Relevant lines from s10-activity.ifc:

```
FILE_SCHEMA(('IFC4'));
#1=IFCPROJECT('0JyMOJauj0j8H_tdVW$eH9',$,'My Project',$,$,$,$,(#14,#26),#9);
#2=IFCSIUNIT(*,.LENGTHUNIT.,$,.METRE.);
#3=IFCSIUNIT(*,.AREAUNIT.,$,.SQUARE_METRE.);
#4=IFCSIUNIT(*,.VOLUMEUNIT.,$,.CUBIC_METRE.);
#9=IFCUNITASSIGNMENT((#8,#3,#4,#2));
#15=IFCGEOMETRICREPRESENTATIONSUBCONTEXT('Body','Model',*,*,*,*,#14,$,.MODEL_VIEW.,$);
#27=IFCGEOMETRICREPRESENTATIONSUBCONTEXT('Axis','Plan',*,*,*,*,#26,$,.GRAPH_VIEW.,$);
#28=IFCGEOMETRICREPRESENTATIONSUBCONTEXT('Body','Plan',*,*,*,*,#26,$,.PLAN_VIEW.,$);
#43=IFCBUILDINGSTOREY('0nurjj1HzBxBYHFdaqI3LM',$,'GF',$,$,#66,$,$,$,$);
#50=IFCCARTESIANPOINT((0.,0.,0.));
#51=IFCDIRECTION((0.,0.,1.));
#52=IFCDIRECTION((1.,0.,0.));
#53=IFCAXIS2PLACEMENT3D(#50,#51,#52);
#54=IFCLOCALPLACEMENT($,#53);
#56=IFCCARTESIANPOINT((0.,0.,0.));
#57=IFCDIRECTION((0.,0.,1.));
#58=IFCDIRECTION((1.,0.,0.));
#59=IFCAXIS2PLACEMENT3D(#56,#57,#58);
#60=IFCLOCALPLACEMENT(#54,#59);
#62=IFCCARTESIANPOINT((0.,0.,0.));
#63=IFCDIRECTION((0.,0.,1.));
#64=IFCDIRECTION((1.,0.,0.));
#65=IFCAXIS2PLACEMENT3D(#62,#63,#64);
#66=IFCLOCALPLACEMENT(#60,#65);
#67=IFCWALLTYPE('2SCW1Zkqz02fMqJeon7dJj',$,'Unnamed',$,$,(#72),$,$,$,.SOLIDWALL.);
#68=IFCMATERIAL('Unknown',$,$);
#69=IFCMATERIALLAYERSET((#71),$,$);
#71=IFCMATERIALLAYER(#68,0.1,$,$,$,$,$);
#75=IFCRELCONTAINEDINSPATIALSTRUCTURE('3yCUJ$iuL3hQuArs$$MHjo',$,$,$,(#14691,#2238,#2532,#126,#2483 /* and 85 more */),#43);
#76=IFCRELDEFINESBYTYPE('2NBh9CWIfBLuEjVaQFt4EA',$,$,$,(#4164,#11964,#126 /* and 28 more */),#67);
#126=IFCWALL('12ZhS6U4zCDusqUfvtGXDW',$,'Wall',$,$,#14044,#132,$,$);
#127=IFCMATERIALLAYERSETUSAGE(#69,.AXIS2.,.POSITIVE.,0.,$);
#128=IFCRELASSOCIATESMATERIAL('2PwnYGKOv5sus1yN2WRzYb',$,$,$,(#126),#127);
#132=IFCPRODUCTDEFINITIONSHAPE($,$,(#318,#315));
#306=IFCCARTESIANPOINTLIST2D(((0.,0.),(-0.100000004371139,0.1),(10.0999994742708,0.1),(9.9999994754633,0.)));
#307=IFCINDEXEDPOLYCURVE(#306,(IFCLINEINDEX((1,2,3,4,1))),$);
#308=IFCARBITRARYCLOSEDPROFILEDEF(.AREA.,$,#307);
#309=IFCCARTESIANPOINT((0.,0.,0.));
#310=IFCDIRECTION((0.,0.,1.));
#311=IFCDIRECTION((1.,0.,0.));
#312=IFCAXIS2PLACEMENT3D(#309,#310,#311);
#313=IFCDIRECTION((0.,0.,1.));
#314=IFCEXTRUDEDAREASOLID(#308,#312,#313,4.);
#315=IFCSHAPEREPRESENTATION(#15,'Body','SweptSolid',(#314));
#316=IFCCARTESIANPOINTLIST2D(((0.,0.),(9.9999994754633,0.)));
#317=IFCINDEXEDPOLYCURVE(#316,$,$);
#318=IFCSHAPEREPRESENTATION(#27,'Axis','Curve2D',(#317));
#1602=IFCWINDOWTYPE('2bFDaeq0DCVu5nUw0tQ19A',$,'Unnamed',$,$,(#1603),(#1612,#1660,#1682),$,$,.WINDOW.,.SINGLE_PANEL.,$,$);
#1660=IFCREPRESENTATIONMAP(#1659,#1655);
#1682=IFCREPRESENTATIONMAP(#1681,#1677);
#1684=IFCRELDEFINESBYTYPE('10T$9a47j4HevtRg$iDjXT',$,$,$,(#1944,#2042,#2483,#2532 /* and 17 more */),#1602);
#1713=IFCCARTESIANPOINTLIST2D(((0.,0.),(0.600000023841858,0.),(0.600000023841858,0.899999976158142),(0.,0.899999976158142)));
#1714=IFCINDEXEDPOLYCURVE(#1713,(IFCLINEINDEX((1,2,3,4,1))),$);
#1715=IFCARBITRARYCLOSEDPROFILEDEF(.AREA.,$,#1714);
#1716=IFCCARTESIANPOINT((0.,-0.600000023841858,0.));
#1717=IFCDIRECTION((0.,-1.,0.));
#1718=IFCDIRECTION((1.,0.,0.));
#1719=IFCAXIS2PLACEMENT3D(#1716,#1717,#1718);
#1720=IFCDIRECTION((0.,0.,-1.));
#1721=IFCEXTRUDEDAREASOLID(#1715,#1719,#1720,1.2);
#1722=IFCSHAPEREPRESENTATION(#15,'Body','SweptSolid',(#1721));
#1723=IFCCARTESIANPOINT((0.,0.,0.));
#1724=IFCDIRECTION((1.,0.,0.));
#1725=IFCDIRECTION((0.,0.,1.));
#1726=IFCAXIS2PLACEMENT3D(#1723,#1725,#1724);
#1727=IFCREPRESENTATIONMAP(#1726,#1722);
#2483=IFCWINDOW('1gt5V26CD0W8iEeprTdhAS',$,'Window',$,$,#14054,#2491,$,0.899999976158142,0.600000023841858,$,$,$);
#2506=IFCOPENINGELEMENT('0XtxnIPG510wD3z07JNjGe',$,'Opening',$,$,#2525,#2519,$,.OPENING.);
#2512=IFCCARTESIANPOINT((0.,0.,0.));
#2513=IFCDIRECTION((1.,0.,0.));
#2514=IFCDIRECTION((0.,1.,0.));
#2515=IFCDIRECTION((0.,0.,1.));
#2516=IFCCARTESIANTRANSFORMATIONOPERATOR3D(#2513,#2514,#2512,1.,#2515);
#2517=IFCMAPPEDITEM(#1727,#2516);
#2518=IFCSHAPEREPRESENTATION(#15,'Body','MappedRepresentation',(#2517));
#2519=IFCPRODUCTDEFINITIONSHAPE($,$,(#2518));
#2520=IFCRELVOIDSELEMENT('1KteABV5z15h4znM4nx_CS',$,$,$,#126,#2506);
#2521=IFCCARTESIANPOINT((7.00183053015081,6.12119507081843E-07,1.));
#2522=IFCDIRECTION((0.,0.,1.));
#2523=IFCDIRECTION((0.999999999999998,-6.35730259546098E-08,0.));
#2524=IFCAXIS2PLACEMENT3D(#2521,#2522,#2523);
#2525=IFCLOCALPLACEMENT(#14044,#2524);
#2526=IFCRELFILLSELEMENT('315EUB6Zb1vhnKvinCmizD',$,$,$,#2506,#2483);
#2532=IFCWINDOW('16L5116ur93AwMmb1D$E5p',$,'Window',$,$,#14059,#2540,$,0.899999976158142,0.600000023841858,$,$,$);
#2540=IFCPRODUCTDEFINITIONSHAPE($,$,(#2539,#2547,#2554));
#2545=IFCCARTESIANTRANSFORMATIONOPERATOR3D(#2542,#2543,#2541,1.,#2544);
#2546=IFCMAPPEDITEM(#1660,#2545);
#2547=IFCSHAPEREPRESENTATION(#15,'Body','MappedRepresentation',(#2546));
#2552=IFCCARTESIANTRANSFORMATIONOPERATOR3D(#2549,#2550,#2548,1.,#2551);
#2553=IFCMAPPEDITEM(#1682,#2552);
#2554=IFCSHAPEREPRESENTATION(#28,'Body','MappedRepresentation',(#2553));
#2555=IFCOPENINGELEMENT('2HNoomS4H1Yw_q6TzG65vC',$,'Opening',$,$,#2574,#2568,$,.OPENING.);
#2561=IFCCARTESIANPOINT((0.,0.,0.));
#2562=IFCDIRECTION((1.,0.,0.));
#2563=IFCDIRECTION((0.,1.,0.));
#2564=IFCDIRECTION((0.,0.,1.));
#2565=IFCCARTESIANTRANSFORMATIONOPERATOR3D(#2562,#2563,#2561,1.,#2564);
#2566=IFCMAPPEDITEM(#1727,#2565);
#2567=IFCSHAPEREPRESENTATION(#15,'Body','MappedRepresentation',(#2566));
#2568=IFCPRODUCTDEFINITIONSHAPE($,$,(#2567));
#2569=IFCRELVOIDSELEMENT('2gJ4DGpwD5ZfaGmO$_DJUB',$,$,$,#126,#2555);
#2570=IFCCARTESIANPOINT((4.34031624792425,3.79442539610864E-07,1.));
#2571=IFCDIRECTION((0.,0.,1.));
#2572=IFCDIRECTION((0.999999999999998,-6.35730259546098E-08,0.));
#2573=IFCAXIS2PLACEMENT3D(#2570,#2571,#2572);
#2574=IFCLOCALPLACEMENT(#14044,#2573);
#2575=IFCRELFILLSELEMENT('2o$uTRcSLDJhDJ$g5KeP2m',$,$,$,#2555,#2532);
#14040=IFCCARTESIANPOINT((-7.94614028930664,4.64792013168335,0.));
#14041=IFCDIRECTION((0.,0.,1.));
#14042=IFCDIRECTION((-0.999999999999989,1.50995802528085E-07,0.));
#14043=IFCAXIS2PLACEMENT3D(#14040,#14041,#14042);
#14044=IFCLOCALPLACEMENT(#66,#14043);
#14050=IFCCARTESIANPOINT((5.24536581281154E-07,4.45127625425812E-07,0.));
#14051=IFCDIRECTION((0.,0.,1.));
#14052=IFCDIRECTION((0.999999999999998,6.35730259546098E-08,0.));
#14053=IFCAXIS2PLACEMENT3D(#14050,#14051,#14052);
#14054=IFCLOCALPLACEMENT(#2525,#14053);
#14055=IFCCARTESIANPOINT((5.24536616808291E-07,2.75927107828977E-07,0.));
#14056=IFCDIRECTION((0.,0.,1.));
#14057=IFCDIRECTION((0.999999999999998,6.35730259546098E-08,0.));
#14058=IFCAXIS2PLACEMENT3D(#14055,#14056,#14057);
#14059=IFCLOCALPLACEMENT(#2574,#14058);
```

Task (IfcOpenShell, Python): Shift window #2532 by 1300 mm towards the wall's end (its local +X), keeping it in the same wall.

```python
import ifcopenshell
import ifcopenshell.api.geometry
import ifcopenshell.util.placement

model = ifcopenshell.open("s10-activity.ifc")

window = model.by_id(2532)
opening = window.FillsVoids[0].RelatingOpeningElement
wall = opening.VoidsElements[0].RelatingBuildingElement

wall_matrix = ifcopenshell.util.placement.get_local_placement(wall.ObjectPlacement)
shift = wall_matrix[:3, 0] * 1.3
before = ifcopenshell.util.placement.get_local_placement(window.ObjectPlacement)[:3, 3].copy()

# The window is placed relative to its opening, so it follows when the opening moves.
matrix = ifcopenshell.util.placement.get_local_placement(opening.ObjectPlacement)
matrix[:3, 3] += shift
ifcopenshell.api.geometry.edit_object_placement(
    model, product=opening, matrix=matrix, is_si=False, should_transform_children=True
)

after = ifcopenshell.util.placement.get_local_placement(window.ObjectPlacement)[:3, 3]
print("window moved by", (after - before).round(3) + 0.0)

model.write("s10-activity-out.ifc")
```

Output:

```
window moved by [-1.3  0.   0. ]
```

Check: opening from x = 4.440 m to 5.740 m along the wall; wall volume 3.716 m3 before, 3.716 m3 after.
